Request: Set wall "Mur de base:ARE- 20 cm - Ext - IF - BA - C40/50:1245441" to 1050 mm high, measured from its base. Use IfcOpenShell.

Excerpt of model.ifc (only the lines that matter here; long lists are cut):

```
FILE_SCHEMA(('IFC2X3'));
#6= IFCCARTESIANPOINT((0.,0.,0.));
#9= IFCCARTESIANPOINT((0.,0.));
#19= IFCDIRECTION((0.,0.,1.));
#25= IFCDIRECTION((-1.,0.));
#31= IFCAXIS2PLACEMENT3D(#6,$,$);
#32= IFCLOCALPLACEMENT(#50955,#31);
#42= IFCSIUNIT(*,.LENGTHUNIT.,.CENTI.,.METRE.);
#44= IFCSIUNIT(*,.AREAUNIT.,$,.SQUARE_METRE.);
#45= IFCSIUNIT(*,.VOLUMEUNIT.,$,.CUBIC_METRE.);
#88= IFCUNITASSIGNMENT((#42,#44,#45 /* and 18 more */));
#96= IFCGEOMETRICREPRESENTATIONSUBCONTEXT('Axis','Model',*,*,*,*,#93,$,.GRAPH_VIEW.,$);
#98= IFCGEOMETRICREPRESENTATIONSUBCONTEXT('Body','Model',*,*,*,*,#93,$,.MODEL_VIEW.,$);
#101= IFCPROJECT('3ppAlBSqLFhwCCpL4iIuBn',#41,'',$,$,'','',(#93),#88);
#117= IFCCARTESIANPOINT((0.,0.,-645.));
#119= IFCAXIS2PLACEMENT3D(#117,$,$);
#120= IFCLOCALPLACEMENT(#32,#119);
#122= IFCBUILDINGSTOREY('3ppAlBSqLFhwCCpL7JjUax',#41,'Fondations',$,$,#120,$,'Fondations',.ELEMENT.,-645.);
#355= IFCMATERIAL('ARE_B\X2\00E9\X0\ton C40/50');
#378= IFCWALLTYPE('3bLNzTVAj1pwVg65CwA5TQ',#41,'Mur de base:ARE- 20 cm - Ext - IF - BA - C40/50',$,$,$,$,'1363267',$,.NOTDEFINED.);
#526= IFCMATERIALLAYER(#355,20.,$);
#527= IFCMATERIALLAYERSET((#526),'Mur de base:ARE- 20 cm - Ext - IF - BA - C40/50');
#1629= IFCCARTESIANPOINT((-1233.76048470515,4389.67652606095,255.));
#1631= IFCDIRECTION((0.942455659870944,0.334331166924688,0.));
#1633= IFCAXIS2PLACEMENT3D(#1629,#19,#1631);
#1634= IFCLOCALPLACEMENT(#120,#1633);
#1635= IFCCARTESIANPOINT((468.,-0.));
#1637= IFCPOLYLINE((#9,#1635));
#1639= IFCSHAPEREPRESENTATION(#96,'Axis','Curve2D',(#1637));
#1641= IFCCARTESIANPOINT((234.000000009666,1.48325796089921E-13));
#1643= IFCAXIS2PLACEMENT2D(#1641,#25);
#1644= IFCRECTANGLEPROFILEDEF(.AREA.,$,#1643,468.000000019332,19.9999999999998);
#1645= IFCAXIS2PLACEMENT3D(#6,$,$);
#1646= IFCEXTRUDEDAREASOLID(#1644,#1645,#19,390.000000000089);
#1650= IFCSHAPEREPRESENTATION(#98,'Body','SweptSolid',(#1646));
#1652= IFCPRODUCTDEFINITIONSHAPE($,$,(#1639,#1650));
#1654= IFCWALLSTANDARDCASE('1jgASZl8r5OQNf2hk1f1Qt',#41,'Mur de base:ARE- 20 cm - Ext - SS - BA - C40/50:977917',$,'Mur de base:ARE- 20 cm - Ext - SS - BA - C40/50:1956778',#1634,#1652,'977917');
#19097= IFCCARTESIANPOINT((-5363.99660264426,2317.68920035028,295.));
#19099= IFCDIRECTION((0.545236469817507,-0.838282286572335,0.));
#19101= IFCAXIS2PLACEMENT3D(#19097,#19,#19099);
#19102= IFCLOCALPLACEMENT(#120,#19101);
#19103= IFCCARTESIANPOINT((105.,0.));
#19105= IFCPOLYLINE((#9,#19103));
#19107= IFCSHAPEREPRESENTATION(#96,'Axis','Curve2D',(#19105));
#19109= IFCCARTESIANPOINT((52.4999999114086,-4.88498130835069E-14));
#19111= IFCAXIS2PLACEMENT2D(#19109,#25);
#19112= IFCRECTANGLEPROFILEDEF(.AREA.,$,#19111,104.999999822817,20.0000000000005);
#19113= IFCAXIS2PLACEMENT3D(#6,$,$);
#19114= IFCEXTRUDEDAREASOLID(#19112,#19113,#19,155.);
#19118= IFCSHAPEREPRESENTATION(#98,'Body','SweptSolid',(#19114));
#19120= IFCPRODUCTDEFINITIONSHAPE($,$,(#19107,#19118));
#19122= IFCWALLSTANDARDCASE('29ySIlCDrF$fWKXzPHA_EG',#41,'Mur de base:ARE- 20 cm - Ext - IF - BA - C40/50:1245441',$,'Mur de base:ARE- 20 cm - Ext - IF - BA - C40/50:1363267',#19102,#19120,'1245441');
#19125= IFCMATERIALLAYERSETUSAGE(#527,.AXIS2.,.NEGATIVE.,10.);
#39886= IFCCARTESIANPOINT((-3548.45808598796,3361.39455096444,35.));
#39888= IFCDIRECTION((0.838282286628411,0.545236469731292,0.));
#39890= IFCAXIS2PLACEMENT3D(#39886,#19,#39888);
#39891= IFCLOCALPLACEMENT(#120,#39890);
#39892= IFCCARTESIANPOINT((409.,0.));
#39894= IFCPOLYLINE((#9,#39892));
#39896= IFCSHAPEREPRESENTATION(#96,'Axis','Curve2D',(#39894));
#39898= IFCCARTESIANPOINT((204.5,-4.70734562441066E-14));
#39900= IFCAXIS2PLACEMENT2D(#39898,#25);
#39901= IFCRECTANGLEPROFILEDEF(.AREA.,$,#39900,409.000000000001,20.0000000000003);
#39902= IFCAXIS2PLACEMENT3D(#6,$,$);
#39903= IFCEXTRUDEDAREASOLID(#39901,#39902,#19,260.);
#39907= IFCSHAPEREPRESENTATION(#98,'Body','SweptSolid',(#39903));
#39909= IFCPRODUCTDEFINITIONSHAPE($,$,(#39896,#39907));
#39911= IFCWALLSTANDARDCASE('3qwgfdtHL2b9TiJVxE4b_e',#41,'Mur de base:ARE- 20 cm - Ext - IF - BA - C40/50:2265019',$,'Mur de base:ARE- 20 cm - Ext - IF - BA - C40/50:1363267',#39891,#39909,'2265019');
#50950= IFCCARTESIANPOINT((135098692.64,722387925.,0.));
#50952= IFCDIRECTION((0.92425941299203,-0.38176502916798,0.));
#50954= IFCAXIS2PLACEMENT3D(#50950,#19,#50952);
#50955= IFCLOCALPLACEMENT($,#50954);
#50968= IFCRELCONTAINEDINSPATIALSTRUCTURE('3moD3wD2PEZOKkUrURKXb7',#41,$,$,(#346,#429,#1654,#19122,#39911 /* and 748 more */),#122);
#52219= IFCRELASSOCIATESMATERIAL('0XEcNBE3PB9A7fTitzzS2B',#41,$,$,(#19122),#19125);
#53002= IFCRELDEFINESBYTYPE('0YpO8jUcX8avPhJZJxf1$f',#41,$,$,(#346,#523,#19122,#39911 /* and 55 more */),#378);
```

```python
import ifcopenshell
import ifcopenshell.geom
import ifcopenshell.util.representation
import ifcopenshell.util.shape
import ifcopenshell.util.unit

model = ifcopenshell.open("model.ifc")
unit_scale = ifcopenshell.util.unit.calculate_unit_scale(model)
settings = ifcopenshell.geom.settings()


def volume(element):
    """Net volume in cubic metres, openings subtracted."""
    shape = ifcopenshell.geom.create_shape(settings, element)
    return ifcopenshell.util.shape.get_volume(shape.geometry)


wall = model.by_guid("29ySIlCDrF$fWKXzPHA_EG")
before = volume(wall)

body = ifcopenshell.util.representation.get_representation(wall, "Model", "Body")
solid = body.Items[0]
old_height = solid.Depth
solid.Depth = 1.05 / unit_scale
after = volume(wall)

print(f"height {old_height:g} -> {solid.Depth:g}, volume {before:.3f} -> {after:.3f} m3")

model.write("model_rev.ifc")
```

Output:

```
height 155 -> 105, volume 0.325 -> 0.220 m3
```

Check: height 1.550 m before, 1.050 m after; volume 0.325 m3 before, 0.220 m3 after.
